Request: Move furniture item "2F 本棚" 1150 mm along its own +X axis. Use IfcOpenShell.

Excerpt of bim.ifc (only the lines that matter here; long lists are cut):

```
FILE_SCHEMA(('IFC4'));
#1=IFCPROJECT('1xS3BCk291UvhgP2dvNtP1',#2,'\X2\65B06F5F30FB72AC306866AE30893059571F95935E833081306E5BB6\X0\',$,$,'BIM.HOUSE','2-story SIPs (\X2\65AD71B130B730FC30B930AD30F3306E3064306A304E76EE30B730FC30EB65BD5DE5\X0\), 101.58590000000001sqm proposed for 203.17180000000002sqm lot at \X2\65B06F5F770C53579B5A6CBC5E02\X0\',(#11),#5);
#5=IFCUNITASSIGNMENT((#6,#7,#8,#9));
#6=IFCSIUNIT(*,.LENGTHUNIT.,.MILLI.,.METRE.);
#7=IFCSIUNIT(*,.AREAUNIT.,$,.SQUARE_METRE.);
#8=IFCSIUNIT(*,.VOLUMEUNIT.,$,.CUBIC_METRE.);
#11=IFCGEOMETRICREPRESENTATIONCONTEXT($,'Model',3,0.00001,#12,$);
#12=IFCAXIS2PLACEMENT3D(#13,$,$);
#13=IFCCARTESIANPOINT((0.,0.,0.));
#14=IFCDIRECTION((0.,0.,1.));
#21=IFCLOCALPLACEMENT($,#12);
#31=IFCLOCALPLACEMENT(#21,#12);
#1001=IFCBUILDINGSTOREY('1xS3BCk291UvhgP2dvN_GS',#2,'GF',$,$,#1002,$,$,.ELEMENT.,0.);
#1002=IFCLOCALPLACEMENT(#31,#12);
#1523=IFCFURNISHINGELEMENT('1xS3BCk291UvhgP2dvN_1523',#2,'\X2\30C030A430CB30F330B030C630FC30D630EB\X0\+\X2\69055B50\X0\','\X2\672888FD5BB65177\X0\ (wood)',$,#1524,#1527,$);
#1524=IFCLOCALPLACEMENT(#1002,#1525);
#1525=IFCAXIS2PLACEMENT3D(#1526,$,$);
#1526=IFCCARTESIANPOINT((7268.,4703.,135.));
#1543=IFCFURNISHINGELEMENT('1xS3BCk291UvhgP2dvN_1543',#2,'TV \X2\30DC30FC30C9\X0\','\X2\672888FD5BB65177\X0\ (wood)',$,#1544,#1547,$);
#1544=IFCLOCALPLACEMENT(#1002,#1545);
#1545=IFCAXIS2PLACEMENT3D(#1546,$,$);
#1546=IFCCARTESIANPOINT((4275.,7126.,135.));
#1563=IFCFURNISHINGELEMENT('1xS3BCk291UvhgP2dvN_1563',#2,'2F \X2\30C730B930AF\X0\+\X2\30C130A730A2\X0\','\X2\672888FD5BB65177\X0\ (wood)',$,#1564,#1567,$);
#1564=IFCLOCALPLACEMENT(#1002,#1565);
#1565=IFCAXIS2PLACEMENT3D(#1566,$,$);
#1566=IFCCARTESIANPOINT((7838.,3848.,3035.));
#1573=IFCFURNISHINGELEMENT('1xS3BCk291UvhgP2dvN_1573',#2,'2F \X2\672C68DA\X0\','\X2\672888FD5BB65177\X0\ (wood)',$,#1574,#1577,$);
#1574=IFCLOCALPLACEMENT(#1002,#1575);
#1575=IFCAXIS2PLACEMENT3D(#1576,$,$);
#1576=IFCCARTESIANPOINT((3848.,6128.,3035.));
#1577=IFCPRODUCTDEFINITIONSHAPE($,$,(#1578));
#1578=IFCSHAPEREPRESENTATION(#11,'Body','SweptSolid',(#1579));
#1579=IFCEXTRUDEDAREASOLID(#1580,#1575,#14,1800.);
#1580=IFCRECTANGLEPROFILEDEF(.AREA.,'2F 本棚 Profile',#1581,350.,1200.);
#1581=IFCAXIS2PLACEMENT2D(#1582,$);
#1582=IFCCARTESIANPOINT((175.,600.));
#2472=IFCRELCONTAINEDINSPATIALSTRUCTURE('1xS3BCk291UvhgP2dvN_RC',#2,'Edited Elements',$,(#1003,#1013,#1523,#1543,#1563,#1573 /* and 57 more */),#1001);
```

```python
import ifcopenshell
import ifcopenshell.api.geometry
import ifcopenshell.util.placement
import ifcopenshell.util.unit

model = ifcopenshell.open("bim.ifc")
unit_scale = ifcopenshell.util.unit.calculate_unit_scale(model)

item = model.by_guid("1xS3BCk291UvhgP2dvN_1573")
matrix = ifcopenshell.util.placement.get_local_placement(item.ObjectPlacement)
matrix[:3, 3] += matrix[:3, 0] * 1.15 / unit_scale
ifcopenshell.api.geometry.edit_object_placement(model, product=item, matrix=matrix, is_si=False)

print(ifcopenshell.util.placement.get_local_placement(item.ObjectPlacement).round(3) + 0.0)

model.write("bim-out.ifc")
```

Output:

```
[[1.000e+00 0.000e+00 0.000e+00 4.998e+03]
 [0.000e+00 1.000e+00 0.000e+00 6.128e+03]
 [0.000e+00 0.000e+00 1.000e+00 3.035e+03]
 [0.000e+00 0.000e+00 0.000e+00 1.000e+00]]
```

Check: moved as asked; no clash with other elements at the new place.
